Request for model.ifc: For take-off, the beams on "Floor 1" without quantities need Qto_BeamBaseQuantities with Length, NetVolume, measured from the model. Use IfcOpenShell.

First a look at what the model holds.

```python
import ifcopenshell
import ifcopenshell.util.element
import ifcopenshell.util.unit

model = ifcopenshell.open("model.ifc")
print(model.schema)
for unit_type in ("LENGTHUNIT", "AREAUNIT", "VOLUMEUNIT"):
    print(unit_type, ifcopenshell.util.unit.calculate_unit_scale(model, unit_type))
storey = next(s for s in model.by_type("IfcBuildingStorey") if s.Name == "Floor 1")
beams = [e for e in ifcopenshell.util.element.get_decomposition(storey) if e.is_a("IfcBeam")]
for e in sorted(beams, key=lambda e: e.id()):
    print(e.id(), e.is_a(), e.Name, list(ifcopenshell.util.element.get_psets(e, qtos_only=True)), sep=" | ")
```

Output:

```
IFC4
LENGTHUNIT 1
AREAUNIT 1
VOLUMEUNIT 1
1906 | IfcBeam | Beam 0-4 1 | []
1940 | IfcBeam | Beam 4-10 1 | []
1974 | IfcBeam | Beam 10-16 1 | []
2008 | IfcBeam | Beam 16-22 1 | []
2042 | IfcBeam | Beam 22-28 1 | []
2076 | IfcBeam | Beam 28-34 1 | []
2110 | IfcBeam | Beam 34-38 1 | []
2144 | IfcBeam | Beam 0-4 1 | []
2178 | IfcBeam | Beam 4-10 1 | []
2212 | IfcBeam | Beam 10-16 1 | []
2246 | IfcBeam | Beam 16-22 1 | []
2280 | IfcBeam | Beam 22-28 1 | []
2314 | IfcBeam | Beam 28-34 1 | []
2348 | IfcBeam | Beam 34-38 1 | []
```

```python
import ifcopenshell
import ifcopenshell.api.pset
import ifcopenshell.geom
import ifcopenshell.util.element
import ifcopenshell.util.shape
import ifcopenshell.util.unit

model = ifcopenshell.open("model.ifc")
unit_scale = ifcopenshell.util.unit.calculate_unit_scale(model)
volume_scale = ifcopenshell.util.unit.calculate_unit_scale(model, "VOLUMEUNIT")
settings = ifcopenshell.geom.settings()

storey = next(s for s in model.by_type("IfcBuildingStorey") if s.Name == "Floor 1")
beams = [e for e in ifcopenshell.util.element.get_decomposition(storey) if e.is_a("IfcBeam")]

for e in sorted(beams, key=lambda e: e.id()):
    if ifcopenshell.util.element.get_psets(e, qtos_only=True, should_inherit=False):
        continue
    # Geometry comes back in metres, in the element's own axes.
    shape = ifcopenshell.geom.create_shape(settings, e)
    values = {
        "Length": ifcopenshell.util.shape.get_max_xyz(shape.geometry) / unit_scale,
        "NetVolume": ifcopenshell.util.shape.get_volume(shape.geometry) / volume_scale,
    }
    qto = ifcopenshell.api.pset.add_qto(model, product=e, name="Qto_BeamBaseQuantities")
    ifcopenshell.api.pset.edit_qto(model, qto=qto, properties=values)
    print(e.id(), {k: round(v, 3) for k, v in values.items()})

model.write("model_rev.ifc")
```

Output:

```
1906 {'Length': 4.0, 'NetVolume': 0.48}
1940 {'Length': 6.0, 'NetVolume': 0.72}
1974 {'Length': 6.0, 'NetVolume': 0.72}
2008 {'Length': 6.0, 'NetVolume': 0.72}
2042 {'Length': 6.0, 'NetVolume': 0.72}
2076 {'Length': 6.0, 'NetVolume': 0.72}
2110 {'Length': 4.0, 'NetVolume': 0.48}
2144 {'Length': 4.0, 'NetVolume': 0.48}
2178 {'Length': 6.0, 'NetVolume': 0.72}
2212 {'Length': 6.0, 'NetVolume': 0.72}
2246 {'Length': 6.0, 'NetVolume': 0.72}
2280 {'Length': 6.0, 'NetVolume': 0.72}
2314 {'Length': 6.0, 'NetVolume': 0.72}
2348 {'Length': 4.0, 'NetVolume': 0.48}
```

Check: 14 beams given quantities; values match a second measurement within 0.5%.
